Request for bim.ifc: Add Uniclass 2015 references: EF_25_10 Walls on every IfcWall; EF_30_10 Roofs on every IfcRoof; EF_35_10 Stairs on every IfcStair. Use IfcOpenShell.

First a look at what the model holds.

```python
import ifcopenshell

model = ifcopenshell.open("bim.ifc")
print(model.schema)
print("classifications:", [c.Name for c in model.by_type("IfcClassification")])
for ifc_class in ("IfcDoor", "IfcRoof", "IfcStair", "IfcWall", "IfcWindow"):
    print(ifc_class, len(model.by_type(ifc_class)))
```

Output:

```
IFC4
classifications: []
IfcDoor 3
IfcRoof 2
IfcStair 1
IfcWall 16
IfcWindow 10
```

```python
import ifcopenshell
import ifcopenshell.api.classification

model = ifcopenshell.open("bim.ifc")

system = ifcopenshell.api.classification.add_classification(model, classification="Uniclass 2015")

codes = {
    "IfcWall": ("EF_25_10", "Walls"),
    "IfcRoof": ("EF_30_10", "Roofs"),
    "IfcStair": ("EF_35_10", "Stairs"),
}
for ifc_class, (code, name) in codes.items():
    products = model.by_type(ifc_class)
    ifcopenshell.api.classification.add_reference(
        model, products=products, classification=system, identification=code, name=name
    )
    print(code, len(products))

model.write("bim_edited.ifc")
```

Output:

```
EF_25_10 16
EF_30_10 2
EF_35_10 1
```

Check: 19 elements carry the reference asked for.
